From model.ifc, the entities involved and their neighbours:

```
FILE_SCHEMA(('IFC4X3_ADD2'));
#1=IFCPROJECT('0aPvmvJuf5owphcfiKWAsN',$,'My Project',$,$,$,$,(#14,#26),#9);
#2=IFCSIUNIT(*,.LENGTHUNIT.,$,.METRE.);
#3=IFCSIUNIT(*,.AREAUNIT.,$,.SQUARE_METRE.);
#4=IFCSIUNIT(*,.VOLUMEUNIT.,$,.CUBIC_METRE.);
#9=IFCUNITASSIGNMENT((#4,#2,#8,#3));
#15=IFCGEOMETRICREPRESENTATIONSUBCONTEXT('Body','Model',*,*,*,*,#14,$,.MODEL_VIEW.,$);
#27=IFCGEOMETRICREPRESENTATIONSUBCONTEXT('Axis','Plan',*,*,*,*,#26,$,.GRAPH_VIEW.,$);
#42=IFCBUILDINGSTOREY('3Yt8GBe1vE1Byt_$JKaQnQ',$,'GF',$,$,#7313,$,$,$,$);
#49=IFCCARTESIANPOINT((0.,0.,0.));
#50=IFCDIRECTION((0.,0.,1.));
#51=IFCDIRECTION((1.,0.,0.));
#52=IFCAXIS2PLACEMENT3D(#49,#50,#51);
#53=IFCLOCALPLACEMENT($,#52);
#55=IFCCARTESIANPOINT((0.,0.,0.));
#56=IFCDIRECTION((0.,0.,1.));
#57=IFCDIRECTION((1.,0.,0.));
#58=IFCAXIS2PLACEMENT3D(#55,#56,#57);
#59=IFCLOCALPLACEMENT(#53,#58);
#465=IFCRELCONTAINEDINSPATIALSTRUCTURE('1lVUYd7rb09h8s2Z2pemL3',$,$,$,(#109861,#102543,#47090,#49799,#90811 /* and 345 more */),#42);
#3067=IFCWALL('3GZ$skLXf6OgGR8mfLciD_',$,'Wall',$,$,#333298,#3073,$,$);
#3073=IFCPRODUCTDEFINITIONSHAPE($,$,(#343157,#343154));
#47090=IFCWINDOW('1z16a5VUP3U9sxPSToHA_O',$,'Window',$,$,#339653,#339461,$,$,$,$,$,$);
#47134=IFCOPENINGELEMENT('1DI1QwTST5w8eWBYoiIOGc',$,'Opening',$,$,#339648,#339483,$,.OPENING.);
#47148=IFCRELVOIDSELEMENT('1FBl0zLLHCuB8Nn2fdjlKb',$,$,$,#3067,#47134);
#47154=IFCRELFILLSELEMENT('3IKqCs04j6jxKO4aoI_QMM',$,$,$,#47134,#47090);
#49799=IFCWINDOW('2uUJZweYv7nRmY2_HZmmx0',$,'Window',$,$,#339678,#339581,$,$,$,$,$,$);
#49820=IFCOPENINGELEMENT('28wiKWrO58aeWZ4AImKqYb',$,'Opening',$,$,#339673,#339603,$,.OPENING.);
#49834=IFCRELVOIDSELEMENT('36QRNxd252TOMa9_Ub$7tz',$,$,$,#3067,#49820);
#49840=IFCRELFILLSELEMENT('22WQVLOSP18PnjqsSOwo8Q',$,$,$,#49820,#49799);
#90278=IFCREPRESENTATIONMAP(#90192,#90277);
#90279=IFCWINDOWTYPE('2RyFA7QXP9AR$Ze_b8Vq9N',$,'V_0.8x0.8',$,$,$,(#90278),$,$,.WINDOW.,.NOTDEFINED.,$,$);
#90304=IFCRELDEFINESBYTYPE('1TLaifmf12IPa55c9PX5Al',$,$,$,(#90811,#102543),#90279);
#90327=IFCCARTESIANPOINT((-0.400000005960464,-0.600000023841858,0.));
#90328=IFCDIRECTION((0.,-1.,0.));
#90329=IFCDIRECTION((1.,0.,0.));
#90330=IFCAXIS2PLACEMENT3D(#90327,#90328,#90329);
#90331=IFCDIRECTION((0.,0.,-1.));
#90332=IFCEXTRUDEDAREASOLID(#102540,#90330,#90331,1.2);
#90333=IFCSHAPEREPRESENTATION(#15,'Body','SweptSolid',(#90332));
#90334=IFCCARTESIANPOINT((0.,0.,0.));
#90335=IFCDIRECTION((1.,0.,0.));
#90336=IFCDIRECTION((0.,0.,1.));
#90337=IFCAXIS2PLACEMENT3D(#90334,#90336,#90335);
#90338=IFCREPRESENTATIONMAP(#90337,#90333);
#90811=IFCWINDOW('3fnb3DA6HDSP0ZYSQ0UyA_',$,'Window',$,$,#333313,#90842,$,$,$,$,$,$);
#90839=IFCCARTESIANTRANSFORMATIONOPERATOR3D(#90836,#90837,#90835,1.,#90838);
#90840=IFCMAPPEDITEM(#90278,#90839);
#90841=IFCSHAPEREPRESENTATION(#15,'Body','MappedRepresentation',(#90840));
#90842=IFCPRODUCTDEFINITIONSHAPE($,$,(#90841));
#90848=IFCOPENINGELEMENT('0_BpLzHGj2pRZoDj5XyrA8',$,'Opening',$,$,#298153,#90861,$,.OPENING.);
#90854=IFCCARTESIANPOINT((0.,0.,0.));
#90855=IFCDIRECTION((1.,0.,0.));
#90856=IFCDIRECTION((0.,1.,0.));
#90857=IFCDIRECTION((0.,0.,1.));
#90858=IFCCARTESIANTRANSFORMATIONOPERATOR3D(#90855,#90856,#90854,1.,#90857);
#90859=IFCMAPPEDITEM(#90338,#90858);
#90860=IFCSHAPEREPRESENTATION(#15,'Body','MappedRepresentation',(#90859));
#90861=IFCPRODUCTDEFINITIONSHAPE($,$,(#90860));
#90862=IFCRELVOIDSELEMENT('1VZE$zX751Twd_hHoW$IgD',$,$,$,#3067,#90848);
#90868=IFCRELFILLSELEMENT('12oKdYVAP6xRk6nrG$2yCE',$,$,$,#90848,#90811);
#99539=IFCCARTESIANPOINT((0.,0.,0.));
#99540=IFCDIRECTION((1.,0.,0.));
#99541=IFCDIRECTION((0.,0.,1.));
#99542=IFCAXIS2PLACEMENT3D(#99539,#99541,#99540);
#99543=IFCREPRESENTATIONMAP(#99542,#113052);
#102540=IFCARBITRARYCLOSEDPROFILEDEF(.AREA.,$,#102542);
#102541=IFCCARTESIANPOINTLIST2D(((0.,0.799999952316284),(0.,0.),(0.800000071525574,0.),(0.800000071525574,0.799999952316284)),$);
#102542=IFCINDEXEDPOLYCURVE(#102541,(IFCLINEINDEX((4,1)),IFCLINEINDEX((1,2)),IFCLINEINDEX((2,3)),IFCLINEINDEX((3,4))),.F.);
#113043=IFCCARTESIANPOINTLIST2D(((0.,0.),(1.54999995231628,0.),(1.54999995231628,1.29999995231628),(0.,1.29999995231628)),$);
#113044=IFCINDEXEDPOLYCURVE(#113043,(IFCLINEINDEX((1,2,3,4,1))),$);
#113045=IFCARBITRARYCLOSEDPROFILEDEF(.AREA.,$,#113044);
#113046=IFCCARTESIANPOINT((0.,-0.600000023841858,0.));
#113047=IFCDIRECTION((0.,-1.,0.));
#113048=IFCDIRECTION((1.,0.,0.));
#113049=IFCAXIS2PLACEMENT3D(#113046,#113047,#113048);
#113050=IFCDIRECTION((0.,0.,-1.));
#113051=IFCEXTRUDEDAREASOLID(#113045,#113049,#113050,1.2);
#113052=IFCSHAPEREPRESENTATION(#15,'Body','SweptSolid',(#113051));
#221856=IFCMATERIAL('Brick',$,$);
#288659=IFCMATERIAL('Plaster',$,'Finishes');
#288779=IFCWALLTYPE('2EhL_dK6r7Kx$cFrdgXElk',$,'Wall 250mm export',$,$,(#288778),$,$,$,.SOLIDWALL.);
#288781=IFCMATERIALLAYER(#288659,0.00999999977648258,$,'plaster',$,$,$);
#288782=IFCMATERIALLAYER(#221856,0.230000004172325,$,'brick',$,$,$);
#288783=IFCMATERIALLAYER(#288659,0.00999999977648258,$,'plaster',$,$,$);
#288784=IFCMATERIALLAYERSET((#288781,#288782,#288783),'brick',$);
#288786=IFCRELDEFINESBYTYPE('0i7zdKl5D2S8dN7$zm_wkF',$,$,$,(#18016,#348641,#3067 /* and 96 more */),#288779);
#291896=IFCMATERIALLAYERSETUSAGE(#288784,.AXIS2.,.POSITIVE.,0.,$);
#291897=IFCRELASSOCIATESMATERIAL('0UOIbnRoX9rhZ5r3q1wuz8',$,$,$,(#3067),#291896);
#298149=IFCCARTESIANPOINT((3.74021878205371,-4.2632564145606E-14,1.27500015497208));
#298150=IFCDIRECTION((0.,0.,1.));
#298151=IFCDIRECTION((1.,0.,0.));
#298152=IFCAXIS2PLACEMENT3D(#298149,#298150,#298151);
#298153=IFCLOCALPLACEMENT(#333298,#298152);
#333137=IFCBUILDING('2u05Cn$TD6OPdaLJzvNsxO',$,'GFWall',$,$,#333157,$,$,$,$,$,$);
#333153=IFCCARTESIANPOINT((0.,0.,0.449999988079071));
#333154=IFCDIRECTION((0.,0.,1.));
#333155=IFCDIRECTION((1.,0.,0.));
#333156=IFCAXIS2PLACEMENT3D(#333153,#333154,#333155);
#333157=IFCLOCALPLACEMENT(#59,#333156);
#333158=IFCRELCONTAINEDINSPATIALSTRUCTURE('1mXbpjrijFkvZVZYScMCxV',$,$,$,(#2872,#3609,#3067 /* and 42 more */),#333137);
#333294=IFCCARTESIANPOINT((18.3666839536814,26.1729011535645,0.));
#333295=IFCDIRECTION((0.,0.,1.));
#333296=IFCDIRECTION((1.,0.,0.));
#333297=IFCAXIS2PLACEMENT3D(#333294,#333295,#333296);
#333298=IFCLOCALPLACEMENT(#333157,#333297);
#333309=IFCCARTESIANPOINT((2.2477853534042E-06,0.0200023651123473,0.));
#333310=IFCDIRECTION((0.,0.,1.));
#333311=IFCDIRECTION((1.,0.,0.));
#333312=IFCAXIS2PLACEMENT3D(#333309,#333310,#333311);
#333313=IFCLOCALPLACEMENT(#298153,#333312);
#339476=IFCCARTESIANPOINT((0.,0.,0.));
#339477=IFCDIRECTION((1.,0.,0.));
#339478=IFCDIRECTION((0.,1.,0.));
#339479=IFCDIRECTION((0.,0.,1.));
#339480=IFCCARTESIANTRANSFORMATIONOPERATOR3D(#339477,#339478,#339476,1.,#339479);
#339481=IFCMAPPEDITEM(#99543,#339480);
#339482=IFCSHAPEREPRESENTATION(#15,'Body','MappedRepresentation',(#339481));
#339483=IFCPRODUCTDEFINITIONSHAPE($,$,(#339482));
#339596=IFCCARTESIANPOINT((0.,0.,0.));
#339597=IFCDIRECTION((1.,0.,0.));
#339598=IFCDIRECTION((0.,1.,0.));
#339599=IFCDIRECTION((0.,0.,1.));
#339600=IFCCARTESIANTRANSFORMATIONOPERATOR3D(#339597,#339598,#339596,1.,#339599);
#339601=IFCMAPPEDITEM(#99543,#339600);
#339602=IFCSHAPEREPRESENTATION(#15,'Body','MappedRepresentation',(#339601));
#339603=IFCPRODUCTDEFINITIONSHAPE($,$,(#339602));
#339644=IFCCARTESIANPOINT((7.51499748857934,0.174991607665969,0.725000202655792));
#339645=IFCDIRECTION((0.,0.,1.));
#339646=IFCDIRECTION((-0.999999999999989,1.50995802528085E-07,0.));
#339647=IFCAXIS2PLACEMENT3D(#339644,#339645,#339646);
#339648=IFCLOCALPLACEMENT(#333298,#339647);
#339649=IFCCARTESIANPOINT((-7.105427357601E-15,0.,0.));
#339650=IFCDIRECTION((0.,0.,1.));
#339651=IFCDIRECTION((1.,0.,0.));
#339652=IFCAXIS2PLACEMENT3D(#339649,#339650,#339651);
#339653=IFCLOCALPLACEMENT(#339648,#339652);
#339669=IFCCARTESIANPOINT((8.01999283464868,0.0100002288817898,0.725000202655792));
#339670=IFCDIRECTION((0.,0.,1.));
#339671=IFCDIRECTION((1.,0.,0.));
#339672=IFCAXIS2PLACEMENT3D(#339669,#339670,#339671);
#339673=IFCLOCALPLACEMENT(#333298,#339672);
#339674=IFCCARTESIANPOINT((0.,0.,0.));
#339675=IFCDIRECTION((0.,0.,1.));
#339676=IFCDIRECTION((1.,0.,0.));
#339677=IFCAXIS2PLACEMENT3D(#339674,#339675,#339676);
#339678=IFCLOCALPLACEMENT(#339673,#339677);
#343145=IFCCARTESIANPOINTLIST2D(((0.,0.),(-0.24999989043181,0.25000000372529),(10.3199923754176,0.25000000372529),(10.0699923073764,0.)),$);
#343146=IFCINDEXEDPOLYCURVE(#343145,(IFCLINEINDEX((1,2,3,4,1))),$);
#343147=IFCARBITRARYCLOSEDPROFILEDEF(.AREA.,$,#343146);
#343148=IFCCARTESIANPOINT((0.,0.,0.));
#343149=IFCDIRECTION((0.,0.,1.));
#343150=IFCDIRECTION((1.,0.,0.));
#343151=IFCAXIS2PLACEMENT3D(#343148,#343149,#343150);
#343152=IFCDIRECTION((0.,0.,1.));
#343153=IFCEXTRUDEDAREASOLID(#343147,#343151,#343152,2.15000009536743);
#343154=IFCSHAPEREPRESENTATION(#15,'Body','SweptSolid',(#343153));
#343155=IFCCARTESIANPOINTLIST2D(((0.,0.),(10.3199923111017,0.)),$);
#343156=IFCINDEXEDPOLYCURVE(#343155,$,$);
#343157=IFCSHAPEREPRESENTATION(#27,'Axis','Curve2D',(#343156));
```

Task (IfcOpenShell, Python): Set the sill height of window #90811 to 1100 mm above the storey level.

```python
import numpy as np
import ifcopenshell
import ifcopenshell.api.geometry
import ifcopenshell.geom
import ifcopenshell.util.element
import ifcopenshell.util.placement
import ifcopenshell.util.shape
import ifcopenshell.util.unit

model = ifcopenshell.open("model.ifc")
unit_scale = ifcopenshell.util.unit.calculate_unit_scale(model)

window = model.by_id(90811)
opening = window.FillsVoids[0].RelatingOpeningElement
storey = ifcopenshell.util.element.get_container(window, ifc_class="IfcBuildingStorey")
level = ifcopenshell.util.placement.get_local_placement(storey.ObjectPlacement)[2, 3]

# The opening's origin need not be at the sill, so measure its lowest point.
shape = ifcopenshell.geom.create_shape(ifcopenshell.geom.settings(), opening)
bottom = ifcopenshell.util.shape.get_shape_bottom_elevation(shape, shape.geometry) / unit_scale
dz = level + 1.1 - bottom

shift = np.array([0.0, 0.0, dz])
# The window is placed relative to its opening, so it follows when the opening moves.
matrix = ifcopenshell.util.placement.get_local_placement(opening.ObjectPlacement)
matrix[:3, 3] += shift
ifcopenshell.api.geometry.edit_object_placement(
    model, product=opening, matrix=matrix, is_si=False, should_transform_children=True
)

print(f"moved by {dz * unit_scale:+.3f} m")

model.write("model-out.ifc")
```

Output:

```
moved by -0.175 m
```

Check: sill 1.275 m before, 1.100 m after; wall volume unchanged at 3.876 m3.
